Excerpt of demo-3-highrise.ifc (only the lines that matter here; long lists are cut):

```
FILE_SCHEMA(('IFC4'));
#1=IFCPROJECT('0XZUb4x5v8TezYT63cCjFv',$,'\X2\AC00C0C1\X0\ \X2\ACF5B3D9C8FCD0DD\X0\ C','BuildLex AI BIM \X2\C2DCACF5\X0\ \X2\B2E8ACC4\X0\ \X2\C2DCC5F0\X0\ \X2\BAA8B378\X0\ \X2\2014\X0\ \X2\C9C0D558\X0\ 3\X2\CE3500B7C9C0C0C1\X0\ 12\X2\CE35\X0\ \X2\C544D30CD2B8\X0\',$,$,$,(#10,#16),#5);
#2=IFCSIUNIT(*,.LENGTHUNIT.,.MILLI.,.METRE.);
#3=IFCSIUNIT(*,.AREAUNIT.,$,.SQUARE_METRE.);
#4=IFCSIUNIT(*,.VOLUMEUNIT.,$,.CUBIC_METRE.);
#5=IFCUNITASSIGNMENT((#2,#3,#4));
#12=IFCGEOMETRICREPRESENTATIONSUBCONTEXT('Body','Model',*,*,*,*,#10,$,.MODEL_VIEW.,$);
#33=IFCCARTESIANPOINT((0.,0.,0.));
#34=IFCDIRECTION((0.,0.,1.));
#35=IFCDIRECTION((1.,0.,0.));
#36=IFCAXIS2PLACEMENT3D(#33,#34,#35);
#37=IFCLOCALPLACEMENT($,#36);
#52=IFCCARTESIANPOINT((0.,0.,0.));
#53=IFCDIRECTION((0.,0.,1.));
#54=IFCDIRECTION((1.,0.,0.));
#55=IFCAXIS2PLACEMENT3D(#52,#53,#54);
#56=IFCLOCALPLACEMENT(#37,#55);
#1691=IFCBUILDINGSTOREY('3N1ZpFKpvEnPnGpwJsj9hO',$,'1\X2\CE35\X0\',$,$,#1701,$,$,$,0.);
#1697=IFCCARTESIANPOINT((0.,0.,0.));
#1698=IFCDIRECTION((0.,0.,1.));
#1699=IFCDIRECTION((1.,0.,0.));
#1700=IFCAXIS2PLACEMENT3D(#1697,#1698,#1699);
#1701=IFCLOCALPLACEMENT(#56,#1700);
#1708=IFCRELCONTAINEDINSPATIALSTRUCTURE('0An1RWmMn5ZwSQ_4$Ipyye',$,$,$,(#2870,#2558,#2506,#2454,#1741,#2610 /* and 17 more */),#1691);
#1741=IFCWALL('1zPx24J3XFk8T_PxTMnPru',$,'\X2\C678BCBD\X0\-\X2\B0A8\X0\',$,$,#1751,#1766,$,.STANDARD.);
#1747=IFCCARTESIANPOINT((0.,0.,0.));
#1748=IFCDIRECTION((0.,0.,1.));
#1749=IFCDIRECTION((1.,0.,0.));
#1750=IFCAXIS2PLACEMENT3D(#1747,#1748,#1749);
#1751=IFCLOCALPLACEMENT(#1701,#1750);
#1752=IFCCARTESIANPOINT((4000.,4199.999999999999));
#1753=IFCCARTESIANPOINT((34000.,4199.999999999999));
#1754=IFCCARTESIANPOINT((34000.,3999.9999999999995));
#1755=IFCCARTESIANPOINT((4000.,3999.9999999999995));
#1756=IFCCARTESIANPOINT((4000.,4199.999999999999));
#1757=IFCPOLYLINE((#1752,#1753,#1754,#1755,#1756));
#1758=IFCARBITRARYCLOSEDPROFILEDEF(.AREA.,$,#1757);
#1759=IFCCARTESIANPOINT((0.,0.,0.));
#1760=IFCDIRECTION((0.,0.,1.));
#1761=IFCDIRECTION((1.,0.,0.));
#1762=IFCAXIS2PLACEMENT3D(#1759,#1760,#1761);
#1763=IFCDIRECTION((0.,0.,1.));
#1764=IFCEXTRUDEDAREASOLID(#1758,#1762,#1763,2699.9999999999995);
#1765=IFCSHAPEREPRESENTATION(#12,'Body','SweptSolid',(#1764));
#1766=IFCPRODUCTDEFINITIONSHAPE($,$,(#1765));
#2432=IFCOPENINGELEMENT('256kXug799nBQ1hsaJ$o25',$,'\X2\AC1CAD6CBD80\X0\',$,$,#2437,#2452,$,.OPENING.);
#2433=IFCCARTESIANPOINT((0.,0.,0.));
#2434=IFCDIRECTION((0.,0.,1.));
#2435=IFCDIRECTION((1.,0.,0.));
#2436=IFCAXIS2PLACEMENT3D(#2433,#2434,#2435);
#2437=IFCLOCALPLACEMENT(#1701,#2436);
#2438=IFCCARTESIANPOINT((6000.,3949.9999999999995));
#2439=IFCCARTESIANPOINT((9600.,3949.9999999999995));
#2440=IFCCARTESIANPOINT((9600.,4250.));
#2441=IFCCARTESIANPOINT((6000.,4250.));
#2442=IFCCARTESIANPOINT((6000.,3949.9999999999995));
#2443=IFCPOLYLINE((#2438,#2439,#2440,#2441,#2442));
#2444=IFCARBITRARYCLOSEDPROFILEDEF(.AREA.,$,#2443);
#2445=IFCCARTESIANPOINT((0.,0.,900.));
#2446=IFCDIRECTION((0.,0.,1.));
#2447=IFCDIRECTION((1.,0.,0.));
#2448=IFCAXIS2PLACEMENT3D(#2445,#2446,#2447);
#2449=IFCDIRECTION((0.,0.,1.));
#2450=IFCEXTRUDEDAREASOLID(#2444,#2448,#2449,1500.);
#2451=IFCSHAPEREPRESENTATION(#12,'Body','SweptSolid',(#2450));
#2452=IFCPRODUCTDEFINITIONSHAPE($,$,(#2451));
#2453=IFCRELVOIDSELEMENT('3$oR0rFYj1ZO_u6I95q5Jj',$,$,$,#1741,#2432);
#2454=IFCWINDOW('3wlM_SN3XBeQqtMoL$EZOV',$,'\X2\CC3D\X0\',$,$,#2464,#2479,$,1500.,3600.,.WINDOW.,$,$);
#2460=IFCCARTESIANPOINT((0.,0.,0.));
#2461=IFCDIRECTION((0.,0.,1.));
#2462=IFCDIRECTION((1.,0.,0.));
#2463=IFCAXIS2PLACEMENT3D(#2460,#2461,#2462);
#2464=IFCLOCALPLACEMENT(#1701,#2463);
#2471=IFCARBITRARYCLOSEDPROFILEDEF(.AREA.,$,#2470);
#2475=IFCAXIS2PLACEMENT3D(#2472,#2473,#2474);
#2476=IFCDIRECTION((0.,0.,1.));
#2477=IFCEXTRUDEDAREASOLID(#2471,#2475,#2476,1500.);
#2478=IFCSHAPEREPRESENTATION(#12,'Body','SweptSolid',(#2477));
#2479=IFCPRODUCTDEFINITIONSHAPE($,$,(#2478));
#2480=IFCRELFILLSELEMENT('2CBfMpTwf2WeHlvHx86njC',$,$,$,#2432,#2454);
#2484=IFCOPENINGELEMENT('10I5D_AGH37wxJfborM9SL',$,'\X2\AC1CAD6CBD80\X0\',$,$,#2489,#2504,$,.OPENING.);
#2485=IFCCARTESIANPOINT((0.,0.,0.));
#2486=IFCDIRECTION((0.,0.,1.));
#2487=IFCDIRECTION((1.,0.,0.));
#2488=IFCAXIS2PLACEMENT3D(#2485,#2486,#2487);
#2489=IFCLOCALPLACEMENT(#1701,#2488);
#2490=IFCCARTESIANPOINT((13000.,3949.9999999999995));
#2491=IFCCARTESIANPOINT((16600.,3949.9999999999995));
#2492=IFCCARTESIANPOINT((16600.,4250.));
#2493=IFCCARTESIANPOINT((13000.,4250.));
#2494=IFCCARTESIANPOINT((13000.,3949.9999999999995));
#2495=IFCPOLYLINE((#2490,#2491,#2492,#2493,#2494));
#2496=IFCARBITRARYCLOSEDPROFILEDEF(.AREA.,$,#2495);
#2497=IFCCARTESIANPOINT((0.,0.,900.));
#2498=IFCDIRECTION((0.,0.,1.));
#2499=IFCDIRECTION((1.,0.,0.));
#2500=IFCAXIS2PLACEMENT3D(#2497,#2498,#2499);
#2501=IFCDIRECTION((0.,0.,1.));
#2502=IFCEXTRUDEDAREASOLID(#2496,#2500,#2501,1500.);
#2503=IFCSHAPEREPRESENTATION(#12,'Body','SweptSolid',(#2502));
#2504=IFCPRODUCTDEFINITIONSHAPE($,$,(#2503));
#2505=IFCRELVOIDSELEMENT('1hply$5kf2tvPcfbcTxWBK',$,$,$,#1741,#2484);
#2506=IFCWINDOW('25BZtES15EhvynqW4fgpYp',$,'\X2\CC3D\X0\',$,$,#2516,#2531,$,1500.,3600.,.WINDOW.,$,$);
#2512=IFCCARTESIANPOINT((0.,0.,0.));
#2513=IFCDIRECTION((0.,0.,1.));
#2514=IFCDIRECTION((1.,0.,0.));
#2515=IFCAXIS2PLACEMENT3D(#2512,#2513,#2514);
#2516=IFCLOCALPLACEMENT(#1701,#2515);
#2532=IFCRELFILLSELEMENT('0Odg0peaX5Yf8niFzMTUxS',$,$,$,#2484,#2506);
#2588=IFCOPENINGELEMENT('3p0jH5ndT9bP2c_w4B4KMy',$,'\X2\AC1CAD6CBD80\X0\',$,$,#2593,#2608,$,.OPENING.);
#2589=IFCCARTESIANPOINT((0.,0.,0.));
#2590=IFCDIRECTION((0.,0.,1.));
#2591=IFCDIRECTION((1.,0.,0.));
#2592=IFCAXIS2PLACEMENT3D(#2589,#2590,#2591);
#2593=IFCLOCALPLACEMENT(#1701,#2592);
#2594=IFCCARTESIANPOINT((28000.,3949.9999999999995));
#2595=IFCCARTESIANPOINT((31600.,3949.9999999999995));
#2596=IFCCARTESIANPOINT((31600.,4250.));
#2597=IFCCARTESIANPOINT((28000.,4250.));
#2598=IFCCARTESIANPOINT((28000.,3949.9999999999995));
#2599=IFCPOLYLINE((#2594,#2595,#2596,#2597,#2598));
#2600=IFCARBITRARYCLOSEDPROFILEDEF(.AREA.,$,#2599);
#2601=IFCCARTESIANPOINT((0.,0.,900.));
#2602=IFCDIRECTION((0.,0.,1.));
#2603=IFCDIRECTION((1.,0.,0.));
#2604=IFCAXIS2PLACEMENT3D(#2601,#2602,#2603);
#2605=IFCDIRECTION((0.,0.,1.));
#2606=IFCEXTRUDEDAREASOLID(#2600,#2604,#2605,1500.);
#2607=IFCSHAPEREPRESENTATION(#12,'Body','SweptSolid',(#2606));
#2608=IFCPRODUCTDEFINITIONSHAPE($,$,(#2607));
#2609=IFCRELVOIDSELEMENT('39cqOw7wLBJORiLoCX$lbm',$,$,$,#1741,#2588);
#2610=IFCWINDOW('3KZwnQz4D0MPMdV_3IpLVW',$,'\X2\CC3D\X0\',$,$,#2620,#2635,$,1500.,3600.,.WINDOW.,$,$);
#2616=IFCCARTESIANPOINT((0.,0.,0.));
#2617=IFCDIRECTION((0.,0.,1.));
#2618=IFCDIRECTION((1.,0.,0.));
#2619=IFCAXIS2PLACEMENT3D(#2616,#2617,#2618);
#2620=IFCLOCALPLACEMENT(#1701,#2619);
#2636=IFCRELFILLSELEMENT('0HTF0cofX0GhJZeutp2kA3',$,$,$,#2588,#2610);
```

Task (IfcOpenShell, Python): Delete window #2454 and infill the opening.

```python
import ifcopenshell
import ifcopenshell.api.feature
import ifcopenshell.api.root
import ifcopenshell.geom
import ifcopenshell.util.shape

model = ifcopenshell.open("demo-3-highrise.ifc")
settings = ifcopenshell.geom.settings()


def volume(element):
    """Net volume in cubic metres, openings subtracted."""
    shape = ifcopenshell.geom.create_shape(settings, element)
    return ifcopenshell.util.shape.get_volume(shape.geometry)


window = model.by_guid("3wlM_SN3XBeQqtMoL$EZOV")
opening = window.FillsVoids[0].RelatingOpeningElement
wall = opening.VoidsElements[0].RelatingBuildingElement
before = volume(wall)

ifcopenshell.api.root.remove_product(model, product=window)
ifcopenshell.api.feature.remove_feature(model, feature=opening)

after = volume(wall)

print(f"wall volume {before:.3f} -> {after:.3f} m3")

model.write("demo-3-highrise-out.ifc")
```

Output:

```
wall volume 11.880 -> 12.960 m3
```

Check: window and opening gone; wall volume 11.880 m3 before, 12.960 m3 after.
